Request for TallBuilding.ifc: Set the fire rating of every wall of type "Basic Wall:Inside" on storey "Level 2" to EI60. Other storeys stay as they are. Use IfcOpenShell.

First a look at what the model holds.

```python
import ifcopenshell
import ifcopenshell.util.element

model = ifcopenshell.open("TallBuilding.ifc")
print(model.schema)
storey = next(s for s in model.by_type("IfcBuildingStorey") if s.Name == "Level 2")
walls = [e for e in ifcopenshell.util.element.get_decomposition(storey) if e.is_a("IfcWall")]
seen = {}
for e in walls:
    element_type = ifcopenshell.util.element.get_type(e)
    key = (element_type.Name if element_type != e and element_type else None, ifcopenshell.util.element.get_pset(e, "Pset_WallCommon", "FireRating"))
    seen[key] = seen.get(key, 0) + 1
for (name, value), count in sorted(seen.items(), key=str):
    print(count, "x", name, "|", value)
```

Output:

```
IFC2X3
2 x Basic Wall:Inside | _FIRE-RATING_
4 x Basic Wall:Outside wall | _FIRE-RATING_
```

```python
import ifcopenshell
import ifcopenshell.api.pset
import ifcopenshell.util.element

model = ifcopenshell.open("TallBuilding.ifc")

storey = next(s for s in model.by_type("IfcBuildingStorey") if s.Name == "Level 2")
walls = [e for e in ifcopenshell.util.element.get_decomposition(storey) if e.is_a("IfcWall")]

count = 0
for e in walls:
    element_type = ifcopenshell.util.element.get_type(e)
    if element_type in (None, e) or element_type.Name != "Basic Wall:Inside":
        continue
    # add_pset returns the element's existing set when there is one.
    pset = ifcopenshell.api.pset.add_pset(model, product=e, name="Pset_WallCommon")
    ifcopenshell.api.pset.edit_pset(model, pset=pset, properties={"FireRating": "EI60"})
    count += 1

print(count, "walls updated")

model.write("TallBuilding_v2.ifc")
```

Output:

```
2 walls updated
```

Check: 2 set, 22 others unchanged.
